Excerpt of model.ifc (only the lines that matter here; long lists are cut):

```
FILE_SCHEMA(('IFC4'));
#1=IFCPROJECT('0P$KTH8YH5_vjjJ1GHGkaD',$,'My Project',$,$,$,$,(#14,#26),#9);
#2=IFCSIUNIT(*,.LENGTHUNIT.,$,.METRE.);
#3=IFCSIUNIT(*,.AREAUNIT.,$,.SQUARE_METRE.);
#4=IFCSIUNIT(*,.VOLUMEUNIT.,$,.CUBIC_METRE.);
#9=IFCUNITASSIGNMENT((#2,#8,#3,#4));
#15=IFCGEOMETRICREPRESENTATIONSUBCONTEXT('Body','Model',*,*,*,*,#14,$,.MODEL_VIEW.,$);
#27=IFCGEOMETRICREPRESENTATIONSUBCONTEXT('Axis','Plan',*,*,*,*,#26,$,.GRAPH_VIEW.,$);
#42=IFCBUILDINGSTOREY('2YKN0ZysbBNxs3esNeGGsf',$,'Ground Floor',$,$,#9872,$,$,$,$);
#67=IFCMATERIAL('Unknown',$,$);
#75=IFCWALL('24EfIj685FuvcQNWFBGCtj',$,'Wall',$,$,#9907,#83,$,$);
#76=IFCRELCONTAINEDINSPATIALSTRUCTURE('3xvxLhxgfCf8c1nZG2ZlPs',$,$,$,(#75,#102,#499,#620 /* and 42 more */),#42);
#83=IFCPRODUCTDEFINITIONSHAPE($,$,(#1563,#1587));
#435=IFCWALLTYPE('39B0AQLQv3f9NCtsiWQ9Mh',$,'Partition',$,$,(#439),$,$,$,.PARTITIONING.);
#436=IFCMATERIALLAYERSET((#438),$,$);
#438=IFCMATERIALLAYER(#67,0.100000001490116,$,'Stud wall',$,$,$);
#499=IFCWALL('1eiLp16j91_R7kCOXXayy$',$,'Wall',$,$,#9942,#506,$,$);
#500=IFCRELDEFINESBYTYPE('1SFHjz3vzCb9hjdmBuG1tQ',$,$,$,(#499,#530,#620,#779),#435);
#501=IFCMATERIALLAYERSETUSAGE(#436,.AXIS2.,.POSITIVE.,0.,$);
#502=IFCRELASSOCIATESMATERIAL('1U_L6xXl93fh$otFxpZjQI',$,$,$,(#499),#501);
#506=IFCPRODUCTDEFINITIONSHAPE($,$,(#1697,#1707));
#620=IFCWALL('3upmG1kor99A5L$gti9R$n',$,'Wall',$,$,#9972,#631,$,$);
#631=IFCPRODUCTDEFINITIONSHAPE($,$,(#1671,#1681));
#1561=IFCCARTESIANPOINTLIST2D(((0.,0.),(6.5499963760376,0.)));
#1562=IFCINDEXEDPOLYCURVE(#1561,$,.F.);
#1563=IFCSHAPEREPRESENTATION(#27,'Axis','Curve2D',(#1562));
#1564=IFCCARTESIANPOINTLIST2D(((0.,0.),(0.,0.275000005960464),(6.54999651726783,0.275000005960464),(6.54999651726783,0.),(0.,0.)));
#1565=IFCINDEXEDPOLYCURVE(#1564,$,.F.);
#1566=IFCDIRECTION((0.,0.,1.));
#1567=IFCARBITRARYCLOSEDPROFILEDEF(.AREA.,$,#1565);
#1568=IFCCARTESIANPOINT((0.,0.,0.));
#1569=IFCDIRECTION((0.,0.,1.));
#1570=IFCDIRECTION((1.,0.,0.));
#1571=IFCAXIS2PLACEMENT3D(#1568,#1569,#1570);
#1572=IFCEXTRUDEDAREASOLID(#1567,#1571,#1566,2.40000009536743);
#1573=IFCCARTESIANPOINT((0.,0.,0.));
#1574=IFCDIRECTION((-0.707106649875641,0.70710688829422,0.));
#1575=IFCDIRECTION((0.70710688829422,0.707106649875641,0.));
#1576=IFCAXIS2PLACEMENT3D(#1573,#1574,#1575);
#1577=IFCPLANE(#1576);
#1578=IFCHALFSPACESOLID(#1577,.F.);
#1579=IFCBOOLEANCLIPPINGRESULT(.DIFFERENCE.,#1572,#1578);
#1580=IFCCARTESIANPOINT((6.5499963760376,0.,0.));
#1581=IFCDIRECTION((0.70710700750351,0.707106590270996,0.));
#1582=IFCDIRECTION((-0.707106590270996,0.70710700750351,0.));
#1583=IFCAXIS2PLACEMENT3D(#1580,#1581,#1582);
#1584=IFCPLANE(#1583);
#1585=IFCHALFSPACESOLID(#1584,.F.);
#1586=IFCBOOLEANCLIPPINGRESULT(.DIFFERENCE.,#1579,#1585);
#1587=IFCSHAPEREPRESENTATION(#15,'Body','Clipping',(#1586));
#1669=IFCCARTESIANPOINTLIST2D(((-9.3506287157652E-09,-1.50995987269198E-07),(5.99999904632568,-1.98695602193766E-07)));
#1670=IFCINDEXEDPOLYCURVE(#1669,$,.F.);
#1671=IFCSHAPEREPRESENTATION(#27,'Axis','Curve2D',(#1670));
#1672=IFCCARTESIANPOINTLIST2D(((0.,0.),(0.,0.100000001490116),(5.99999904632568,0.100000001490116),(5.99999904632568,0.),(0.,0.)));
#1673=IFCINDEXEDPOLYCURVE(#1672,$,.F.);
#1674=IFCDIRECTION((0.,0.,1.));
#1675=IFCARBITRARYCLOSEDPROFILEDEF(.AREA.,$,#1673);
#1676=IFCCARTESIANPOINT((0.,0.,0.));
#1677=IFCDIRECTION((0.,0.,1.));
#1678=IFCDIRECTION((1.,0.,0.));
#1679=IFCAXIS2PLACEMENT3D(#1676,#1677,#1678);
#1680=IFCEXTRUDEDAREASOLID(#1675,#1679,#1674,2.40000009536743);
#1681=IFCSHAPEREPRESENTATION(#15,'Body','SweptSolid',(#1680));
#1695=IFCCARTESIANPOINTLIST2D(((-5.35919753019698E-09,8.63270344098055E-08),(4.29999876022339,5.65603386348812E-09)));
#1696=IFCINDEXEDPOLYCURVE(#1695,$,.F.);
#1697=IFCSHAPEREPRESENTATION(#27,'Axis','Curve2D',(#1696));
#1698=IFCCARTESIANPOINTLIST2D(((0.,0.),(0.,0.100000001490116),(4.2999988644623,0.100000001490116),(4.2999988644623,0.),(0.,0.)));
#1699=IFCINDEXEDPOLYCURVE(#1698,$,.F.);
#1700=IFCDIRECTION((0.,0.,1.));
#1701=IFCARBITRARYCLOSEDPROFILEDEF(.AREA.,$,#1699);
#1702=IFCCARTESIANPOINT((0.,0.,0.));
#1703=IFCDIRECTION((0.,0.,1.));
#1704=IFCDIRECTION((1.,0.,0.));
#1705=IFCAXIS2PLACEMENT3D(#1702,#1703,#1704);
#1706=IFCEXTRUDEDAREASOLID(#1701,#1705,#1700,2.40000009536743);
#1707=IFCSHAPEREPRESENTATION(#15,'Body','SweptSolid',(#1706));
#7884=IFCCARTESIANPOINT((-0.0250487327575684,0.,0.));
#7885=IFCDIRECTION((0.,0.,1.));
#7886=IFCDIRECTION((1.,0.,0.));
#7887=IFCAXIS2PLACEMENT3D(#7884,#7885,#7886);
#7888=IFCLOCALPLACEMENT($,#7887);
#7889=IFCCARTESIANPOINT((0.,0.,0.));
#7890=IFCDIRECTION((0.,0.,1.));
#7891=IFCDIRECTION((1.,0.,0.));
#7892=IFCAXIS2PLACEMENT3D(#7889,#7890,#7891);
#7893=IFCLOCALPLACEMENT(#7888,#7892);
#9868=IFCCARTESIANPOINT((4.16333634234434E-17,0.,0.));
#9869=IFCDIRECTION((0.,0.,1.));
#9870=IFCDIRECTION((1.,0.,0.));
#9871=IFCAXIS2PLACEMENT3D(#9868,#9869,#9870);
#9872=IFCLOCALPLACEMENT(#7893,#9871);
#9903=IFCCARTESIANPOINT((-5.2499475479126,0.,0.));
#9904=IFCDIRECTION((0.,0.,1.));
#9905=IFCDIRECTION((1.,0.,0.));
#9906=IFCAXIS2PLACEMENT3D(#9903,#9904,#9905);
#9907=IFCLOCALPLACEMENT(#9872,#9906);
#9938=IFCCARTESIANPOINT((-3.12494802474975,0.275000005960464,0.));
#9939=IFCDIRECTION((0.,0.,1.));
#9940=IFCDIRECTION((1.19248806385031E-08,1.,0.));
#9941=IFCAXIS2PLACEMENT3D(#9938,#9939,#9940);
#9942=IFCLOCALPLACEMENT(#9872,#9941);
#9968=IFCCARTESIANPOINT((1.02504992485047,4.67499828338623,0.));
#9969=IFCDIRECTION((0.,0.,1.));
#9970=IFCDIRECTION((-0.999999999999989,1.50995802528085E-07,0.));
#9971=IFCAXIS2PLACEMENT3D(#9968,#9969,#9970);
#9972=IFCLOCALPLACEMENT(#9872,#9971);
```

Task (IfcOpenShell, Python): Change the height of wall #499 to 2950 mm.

```python
import ifcopenshell
import ifcopenshell.geom
import ifcopenshell.util.representation
import ifcopenshell.util.shape
import ifcopenshell.util.unit

model = ifcopenshell.open("model.ifc")
unit_scale = ifcopenshell.util.unit.calculate_unit_scale(model)
settings = ifcopenshell.geom.settings()


def volume(element):
    """Net volume in cubic metres, openings subtracted."""
    shape = ifcopenshell.geom.create_shape(settings, element)
    return ifcopenshell.util.shape.get_volume(shape.geometry)


wall = model.by_guid("1eiLp16j91_R7kCOXXayy$")
before = volume(wall)

body = ifcopenshell.util.representation.get_representation(wall, "Model", "Body")
solid = body.Items[0]
old_height = solid.Depth
solid.Depth = 2.95 / unit_scale
after = volume(wall)

print(f"height {old_height:g} -> {solid.Depth:g}, volume {before:.3f} -> {after:.3f} m3")

model.write("model-out.ifc")
```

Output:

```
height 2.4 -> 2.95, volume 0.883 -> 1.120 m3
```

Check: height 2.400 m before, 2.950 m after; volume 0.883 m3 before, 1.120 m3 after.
